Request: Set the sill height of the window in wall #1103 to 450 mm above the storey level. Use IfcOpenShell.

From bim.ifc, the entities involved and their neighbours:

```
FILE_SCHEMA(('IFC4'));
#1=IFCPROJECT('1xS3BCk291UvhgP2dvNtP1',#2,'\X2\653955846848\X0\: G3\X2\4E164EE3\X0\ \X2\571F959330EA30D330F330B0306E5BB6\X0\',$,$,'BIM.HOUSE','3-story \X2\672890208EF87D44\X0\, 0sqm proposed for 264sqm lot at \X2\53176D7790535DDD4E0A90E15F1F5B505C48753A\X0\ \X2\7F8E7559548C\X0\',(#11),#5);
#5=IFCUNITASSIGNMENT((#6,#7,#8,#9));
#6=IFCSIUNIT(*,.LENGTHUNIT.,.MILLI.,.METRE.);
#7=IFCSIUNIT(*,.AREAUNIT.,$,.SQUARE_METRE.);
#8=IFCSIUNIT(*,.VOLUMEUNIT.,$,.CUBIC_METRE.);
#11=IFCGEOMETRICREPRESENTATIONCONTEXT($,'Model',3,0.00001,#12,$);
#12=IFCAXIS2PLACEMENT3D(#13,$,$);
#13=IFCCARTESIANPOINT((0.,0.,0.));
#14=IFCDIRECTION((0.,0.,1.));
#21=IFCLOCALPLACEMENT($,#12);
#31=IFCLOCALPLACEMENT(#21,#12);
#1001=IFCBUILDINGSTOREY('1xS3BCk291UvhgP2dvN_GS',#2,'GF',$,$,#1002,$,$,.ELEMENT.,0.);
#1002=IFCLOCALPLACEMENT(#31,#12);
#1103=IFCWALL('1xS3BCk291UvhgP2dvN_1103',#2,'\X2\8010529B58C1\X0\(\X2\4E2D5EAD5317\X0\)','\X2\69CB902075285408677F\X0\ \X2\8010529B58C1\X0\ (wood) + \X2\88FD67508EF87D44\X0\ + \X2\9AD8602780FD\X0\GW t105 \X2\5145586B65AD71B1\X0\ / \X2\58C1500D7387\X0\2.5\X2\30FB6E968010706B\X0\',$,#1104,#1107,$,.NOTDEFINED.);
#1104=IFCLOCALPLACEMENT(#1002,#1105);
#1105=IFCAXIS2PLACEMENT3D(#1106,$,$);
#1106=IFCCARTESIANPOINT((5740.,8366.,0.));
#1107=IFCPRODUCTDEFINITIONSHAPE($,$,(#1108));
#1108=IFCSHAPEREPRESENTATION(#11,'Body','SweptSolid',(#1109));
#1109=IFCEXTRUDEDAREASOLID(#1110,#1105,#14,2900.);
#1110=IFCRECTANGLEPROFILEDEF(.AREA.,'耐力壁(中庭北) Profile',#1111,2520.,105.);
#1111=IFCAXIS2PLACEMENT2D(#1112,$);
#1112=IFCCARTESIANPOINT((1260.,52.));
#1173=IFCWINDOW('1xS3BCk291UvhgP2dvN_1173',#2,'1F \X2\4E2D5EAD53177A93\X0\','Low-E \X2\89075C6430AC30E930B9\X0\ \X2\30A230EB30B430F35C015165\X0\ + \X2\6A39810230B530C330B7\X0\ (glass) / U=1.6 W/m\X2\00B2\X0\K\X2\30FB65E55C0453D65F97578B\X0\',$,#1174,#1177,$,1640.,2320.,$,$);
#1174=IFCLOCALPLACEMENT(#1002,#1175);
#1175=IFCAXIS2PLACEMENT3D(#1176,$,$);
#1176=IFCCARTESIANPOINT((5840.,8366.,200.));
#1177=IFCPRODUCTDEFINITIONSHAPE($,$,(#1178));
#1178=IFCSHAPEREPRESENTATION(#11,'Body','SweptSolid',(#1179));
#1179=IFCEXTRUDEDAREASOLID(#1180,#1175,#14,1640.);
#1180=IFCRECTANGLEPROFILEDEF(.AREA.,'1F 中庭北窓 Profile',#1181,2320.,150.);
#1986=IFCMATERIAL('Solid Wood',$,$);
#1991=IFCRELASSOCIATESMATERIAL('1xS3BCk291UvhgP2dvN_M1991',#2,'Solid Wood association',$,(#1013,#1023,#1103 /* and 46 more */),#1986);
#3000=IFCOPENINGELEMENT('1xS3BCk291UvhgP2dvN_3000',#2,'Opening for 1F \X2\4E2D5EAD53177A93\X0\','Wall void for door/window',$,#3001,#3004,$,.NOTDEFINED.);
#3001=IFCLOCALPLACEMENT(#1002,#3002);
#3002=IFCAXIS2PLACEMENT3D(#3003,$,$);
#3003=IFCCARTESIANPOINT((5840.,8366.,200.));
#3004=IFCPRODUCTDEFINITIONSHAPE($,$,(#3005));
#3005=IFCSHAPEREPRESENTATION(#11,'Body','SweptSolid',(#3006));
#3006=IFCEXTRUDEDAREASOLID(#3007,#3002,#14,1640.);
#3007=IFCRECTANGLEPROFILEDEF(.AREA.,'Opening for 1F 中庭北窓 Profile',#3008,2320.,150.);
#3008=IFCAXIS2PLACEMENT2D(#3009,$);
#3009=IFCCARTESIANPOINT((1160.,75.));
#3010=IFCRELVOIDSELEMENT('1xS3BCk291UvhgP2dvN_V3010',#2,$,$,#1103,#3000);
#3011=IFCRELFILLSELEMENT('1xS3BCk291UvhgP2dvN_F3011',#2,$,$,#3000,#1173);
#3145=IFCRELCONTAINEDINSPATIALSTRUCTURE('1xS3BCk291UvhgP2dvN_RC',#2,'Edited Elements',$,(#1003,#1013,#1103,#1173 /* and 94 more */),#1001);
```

```python
import numpy as np
import ifcopenshell
import ifcopenshell.api.geometry
import ifcopenshell.geom
import ifcopenshell.util.element
import ifcopenshell.util.placement
import ifcopenshell.util.shape
import ifcopenshell.util.unit

model = ifcopenshell.open("bim.ifc")
unit_scale = ifcopenshell.util.unit.calculate_unit_scale(model)

window = model.by_guid("1xS3BCk291UvhgP2dvN_1173")
opening = window.FillsVoids[0].RelatingOpeningElement
storey = ifcopenshell.util.element.get_container(window, ifc_class="IfcBuildingStorey")
level = ifcopenshell.util.placement.get_local_placement(storey.ObjectPlacement)[2, 3]

# The opening's origin need not be at the sill, so measure its lowest point.
shape = ifcopenshell.geom.create_shape(ifcopenshell.geom.settings(), opening)
bottom = ifcopenshell.util.shape.get_shape_bottom_elevation(shape, shape.geometry) / unit_scale
dz = level + 0.45 / unit_scale - bottom

shift = np.array([0.0, 0.0, dz])
# The window is not placed relative to its opening, so move both.
for product in (opening, window):
    matrix = ifcopenshell.util.placement.get_local_placement(product.ObjectPlacement)
    matrix[:3, 3] += shift
    ifcopenshell.api.geometry.edit_object_placement(model, product=product, matrix=matrix, is_si=False)

print(f"moved by {dz * unit_scale:+.3f} m")

model.write("bim_rev.ifc")
```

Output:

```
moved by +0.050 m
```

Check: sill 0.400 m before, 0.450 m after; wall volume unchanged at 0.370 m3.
